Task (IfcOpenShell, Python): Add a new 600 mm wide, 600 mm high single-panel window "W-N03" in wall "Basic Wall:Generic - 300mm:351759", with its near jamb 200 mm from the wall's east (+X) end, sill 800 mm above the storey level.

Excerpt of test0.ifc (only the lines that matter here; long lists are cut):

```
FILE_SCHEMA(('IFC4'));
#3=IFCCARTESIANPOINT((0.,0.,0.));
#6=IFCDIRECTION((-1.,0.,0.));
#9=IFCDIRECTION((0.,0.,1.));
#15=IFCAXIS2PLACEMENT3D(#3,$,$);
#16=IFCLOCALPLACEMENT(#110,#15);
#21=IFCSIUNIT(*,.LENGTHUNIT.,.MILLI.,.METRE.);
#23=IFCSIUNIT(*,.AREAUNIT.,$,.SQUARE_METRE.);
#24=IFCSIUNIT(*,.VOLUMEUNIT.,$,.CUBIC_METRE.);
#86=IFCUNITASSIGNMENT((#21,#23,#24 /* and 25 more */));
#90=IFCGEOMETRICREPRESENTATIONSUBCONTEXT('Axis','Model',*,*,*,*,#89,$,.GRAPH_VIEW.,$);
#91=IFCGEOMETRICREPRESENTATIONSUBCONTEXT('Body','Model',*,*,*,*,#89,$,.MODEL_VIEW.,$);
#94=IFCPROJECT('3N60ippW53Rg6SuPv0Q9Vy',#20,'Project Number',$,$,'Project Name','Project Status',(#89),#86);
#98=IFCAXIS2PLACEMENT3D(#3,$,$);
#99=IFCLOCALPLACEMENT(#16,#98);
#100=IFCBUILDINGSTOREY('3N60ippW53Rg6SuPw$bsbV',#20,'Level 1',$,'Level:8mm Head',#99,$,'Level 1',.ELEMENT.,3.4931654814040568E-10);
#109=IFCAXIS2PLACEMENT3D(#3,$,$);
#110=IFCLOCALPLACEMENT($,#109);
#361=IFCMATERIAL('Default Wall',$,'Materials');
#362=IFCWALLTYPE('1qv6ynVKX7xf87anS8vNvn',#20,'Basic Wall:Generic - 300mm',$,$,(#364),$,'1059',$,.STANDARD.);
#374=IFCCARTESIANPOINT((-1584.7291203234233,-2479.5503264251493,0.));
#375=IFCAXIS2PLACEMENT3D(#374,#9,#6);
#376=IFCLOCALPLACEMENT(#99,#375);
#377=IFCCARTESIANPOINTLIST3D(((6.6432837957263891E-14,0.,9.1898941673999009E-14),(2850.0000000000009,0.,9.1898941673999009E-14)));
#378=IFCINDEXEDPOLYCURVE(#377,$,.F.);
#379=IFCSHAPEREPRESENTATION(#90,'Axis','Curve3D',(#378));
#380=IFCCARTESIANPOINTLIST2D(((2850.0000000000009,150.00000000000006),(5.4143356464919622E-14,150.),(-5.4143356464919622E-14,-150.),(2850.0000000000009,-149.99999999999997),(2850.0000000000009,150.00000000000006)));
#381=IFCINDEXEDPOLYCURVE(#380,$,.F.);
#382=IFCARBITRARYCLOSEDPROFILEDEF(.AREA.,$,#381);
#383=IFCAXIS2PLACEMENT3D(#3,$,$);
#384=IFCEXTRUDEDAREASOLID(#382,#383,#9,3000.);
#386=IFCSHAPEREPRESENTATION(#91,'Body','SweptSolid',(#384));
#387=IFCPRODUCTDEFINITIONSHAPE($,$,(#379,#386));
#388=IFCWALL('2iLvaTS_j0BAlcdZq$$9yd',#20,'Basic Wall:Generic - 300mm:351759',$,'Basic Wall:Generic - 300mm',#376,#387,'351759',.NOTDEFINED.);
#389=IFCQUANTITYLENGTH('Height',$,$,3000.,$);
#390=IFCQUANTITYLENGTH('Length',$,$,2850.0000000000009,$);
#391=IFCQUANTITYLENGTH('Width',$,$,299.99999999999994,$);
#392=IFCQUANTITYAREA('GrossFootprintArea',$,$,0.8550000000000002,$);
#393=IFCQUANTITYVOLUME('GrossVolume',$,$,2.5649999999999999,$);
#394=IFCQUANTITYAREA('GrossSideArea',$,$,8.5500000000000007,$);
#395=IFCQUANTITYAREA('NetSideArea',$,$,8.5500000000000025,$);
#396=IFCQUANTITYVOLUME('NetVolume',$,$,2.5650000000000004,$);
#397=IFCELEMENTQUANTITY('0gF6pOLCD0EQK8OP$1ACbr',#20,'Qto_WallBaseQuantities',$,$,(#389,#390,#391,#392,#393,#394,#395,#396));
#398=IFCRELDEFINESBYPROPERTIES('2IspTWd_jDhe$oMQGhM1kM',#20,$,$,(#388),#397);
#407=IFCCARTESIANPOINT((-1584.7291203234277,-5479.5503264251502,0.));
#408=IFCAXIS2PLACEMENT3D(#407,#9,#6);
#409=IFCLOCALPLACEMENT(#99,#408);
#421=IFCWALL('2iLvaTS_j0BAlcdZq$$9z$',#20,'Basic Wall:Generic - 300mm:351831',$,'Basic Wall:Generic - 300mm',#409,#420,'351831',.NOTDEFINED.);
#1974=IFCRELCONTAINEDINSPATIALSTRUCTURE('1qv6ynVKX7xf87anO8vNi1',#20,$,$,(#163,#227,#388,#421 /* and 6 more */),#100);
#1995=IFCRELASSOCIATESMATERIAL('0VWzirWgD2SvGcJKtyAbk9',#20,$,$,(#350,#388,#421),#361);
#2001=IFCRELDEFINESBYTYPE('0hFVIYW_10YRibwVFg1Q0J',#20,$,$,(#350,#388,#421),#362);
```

```python
import numpy as np
import ifcopenshell
import ifcopenshell.api.feature
import ifcopenshell.api.geometry
import ifcopenshell.api.pset
import ifcopenshell.api.root
import ifcopenshell.api.spatial
import ifcopenshell.geom
import ifcopenshell.util.element
import ifcopenshell.util.placement
import ifcopenshell.util.representation
import ifcopenshell.util.shape
import ifcopenshell.util.unit

model = ifcopenshell.open("test0.ifc")
unit_scale = ifcopenshell.util.unit.calculate_unit_scale(model)
area_scale = ifcopenshell.util.unit.calculate_unit_scale(model, "AREAUNIT")
volume_scale = ifcopenshell.util.unit.calculate_unit_scale(model, "VOLUMEUNIT")
settings = ifcopenshell.geom.settings()


def volume(element):
    """Net volume in cubic metres, openings subtracted."""
    shape = ifcopenshell.geom.create_shape(settings, element)
    return ifcopenshell.util.shape.get_volume(shape.geometry)


wall = model.by_guid("2iLvaTS_j0BAlcdZq$$9yd")
storey = ifcopenshell.util.element.get_container(wall, ifc_class="IfcBuildingStorey")
context = ifcopenshell.util.representation.get_context(model, "Model", "Body", "MODEL_VIEW")
before = volume(wall)

width, height, from_end, sill = 0.6, 0.6, 0.2, 0.8  # metres

# The wall runs along its own X axis, and the end named is its -X end.
wall_shape = ifcopenshell.geom.create_shape(settings, wall)
x, y, z = ifcopenshell.util.shape.get_vertices(wall_shape.geometry).T
start = x.min() + from_end
face, thickness = float(y.min()), float(y.max() - y.min())
wall_matrix = ifcopenshell.util.placement.get_local_placement(wall.ObjectPlacement)
level = ifcopenshell.util.placement.get_local_placement(storey.ObjectPlacement)[2, 3]


def in_wall(x, y):
    """Placement at x, y metres in the wall's axes, at sill height."""
    matrix = wall_matrix.copy()
    matrix[:, 3] = wall_matrix @ np.array([x / unit_scale, y / unit_scale, 0.0, 1.0])
    matrix[2, 3] = level + sill / unit_scale
    return matrix


# Opening: a box that overshoots both wall faces by 50 mm.
opening = ifcopenshell.api.root.create_entity(model, ifc_class="IfcOpeningElement", predefined_type="OPENING")
box = ifcopenshell.api.geometry.add_wall_representation(
    model, context=context, length=width, height=height, thickness=thickness + 0.1
)
ifcopenshell.api.geometry.assign_representation(model, product=opening, representation=box)
ifcopenshell.api.geometry.edit_object_placement(model, product=opening, matrix=in_wall(start, face - 0.05), is_si=False)
ifcopenshell.api.feature.add_feature(model, feature=opening, element=wall)

window = ifcopenshell.api.root.create_entity(model, ifc_class="IfcWindow", name="W-N03", predefined_type="WINDOW")
window.OverallWidth, window.OverallHeight = width / unit_scale, height / unit_scale
window.PartitioningType = "SINGLE_PANEL"
body = ifcopenshell.api.geometry.add_window_representation(
    model,
    context=context,
    overall_width=window.OverallWidth,
    overall_height=window.OverallHeight,
    partition_type="SINGLE_PANEL",
)
ifcopenshell.api.geometry.assign_representation(model, product=window, representation=body)
ifcopenshell.api.spatial.assign_container(model, products=[window], relating_structure=storey)
ifcopenshell.api.feature.add_filling(model, opening=opening, element=window)

# Centre the window in the wall's thickness.
ifcopenshell.api.geometry.edit_object_placement(model, product=window, matrix=in_wall(start, face), is_si=False)
window_shape = ifcopenshell.geom.create_shape(settings, window)
depth = ifcopenshell.util.shape.get_vertices(window_shape.geometry)[:, 1]
offset = face + thickness / 2 - (depth.min() + depth.max()) / 2
ifcopenshell.api.geometry.edit_object_placement(model, product=window, matrix=in_wall(start, offset), is_si=False)

after = volume(wall)

# Update the wall's stored quantities.
qto = model.by_id(ifcopenshell.util.element.get_pset(wall, "Qto_WallBaseQuantities", should_inherit=False)["id"])
ifcopenshell.api.pset.edit_qto(model, qto=qto, properties={
    "NetSideArea": after / thickness / area_scale,
    "NetVolume": after / volume_scale,
})

print(f"wall volume {before:.3f} -> {after:.3f} m3")

model.write("test0-out.ifc")
```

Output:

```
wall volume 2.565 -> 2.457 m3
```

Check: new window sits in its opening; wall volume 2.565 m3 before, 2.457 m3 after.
